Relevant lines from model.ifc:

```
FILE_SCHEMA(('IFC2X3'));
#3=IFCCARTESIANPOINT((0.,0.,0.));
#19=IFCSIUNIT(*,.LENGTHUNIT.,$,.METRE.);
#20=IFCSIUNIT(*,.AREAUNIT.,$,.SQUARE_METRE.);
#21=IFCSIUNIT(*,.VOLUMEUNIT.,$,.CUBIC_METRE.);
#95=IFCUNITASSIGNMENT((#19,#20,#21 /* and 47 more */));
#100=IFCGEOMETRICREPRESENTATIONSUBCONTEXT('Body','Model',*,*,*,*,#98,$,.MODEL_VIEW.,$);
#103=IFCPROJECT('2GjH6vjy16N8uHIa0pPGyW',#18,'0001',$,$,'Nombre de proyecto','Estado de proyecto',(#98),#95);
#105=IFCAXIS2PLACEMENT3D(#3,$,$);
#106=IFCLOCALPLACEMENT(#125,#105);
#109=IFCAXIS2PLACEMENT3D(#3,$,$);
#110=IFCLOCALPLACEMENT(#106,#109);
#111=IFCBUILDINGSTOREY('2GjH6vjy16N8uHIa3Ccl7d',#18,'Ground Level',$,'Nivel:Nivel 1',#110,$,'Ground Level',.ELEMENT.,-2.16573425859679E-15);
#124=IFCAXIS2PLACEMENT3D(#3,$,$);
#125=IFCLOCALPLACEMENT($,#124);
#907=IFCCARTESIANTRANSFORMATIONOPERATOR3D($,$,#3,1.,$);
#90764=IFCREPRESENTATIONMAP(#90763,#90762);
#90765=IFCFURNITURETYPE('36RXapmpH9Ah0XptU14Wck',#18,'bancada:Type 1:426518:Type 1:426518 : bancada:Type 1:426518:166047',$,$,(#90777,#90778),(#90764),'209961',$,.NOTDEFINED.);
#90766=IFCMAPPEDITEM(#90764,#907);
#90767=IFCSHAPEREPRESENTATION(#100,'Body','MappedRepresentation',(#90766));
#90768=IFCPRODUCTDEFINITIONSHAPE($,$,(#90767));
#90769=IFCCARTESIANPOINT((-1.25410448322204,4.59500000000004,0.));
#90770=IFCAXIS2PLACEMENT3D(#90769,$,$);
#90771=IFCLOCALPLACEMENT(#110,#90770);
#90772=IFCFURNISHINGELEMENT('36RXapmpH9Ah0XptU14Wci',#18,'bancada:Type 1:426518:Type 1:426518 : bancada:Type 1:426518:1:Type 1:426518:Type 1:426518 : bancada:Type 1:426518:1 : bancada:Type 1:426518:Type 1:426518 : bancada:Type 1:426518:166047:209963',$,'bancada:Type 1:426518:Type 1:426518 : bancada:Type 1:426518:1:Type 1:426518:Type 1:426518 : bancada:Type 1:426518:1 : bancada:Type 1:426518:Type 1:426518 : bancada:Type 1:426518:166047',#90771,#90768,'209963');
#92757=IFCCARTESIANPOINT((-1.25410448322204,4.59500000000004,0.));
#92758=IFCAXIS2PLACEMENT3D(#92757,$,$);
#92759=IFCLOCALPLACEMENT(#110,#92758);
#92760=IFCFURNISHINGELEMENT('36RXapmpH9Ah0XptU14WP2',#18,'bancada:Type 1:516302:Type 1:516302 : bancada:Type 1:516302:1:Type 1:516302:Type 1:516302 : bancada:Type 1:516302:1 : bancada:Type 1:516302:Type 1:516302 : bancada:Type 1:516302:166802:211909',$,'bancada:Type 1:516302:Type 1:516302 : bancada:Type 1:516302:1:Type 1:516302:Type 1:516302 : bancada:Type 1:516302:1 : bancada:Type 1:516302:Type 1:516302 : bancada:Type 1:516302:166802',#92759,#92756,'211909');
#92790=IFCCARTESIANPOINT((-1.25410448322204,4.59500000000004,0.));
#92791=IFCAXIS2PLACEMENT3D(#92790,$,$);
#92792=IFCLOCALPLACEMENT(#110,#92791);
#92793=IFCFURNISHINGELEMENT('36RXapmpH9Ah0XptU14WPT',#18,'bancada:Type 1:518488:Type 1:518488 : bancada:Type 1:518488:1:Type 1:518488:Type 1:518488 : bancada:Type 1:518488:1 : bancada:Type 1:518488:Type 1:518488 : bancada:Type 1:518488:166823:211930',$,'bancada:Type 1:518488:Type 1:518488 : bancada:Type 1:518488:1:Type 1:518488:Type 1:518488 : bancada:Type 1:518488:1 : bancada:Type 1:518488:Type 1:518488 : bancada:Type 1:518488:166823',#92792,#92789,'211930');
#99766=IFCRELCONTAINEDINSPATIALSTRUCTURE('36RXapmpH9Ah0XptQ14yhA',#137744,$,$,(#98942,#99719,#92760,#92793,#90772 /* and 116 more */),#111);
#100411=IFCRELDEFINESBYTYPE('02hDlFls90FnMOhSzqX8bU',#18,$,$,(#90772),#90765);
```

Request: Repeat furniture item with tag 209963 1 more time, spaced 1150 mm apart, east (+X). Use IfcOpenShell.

```python
import numpy as np
import ifcopenshell
import ifcopenshell.api.geometry
import ifcopenshell.api.root
import ifcopenshell.util.element
import ifcopenshell.util.placement
import ifcopenshell.util.unit

model = ifcopenshell.open("model.ifc")
unit_scale = ifcopenshell.util.unit.calculate_unit_scale(model)


def reuse_history(source, copy):
    """copy_class also copies each property set's owner history, people and application; keep the originals."""
    for rel in copy.IsDefinedBy:
        if rel.is_a("IfcRelDefinesByProperties") and (history := rel.RelatingPropertyDefinition.OwnerHistory):
            rel.RelatingPropertyDefinition.OwnerHistory = source.OwnerHistory
            ifcopenshell.util.element.remove_deep2(model, history)


source = model.by_guid("36RXapmpH9Ah0XptU14Wci")
base = ifcopenshell.util.placement.get_local_placement(source.ObjectPlacement)
step = np.array([1.0, 0.0, 0.0]) * 1.15 / unit_scale

for i in range(1, 2):
    copy = ifcopenshell.api.root.copy_class(model, product=source)
    copy.Representation = ifcopenshell.util.element.copy_deep(
        model, source.Representation, exclude=["IfcGeometricRepresentationContext", "IfcRepresentationMap"]
    )
    copy.Name = "bancada:Type 1:426518:Type 1:426518 : bancada:Type 1:426518:1:Type 1:426518:Type 1:426518 : bancada:Type 1:426518:1 : bancada:Type 1:426518:Type 1:426518 : bancada:Type 1:426518"
    copy.Tag = None
    reuse_history(source, copy)
    matrix = base.copy()
    matrix[:3, 3] += i * step
    print("added at", matrix[:3, 3].round(3) + 0.0)
    ifcopenshell.api.geometry.edit_object_placement(model, product=copy, matrix=matrix, is_si=False)

model.write("model-out.ifc")
```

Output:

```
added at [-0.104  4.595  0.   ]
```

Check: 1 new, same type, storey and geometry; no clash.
